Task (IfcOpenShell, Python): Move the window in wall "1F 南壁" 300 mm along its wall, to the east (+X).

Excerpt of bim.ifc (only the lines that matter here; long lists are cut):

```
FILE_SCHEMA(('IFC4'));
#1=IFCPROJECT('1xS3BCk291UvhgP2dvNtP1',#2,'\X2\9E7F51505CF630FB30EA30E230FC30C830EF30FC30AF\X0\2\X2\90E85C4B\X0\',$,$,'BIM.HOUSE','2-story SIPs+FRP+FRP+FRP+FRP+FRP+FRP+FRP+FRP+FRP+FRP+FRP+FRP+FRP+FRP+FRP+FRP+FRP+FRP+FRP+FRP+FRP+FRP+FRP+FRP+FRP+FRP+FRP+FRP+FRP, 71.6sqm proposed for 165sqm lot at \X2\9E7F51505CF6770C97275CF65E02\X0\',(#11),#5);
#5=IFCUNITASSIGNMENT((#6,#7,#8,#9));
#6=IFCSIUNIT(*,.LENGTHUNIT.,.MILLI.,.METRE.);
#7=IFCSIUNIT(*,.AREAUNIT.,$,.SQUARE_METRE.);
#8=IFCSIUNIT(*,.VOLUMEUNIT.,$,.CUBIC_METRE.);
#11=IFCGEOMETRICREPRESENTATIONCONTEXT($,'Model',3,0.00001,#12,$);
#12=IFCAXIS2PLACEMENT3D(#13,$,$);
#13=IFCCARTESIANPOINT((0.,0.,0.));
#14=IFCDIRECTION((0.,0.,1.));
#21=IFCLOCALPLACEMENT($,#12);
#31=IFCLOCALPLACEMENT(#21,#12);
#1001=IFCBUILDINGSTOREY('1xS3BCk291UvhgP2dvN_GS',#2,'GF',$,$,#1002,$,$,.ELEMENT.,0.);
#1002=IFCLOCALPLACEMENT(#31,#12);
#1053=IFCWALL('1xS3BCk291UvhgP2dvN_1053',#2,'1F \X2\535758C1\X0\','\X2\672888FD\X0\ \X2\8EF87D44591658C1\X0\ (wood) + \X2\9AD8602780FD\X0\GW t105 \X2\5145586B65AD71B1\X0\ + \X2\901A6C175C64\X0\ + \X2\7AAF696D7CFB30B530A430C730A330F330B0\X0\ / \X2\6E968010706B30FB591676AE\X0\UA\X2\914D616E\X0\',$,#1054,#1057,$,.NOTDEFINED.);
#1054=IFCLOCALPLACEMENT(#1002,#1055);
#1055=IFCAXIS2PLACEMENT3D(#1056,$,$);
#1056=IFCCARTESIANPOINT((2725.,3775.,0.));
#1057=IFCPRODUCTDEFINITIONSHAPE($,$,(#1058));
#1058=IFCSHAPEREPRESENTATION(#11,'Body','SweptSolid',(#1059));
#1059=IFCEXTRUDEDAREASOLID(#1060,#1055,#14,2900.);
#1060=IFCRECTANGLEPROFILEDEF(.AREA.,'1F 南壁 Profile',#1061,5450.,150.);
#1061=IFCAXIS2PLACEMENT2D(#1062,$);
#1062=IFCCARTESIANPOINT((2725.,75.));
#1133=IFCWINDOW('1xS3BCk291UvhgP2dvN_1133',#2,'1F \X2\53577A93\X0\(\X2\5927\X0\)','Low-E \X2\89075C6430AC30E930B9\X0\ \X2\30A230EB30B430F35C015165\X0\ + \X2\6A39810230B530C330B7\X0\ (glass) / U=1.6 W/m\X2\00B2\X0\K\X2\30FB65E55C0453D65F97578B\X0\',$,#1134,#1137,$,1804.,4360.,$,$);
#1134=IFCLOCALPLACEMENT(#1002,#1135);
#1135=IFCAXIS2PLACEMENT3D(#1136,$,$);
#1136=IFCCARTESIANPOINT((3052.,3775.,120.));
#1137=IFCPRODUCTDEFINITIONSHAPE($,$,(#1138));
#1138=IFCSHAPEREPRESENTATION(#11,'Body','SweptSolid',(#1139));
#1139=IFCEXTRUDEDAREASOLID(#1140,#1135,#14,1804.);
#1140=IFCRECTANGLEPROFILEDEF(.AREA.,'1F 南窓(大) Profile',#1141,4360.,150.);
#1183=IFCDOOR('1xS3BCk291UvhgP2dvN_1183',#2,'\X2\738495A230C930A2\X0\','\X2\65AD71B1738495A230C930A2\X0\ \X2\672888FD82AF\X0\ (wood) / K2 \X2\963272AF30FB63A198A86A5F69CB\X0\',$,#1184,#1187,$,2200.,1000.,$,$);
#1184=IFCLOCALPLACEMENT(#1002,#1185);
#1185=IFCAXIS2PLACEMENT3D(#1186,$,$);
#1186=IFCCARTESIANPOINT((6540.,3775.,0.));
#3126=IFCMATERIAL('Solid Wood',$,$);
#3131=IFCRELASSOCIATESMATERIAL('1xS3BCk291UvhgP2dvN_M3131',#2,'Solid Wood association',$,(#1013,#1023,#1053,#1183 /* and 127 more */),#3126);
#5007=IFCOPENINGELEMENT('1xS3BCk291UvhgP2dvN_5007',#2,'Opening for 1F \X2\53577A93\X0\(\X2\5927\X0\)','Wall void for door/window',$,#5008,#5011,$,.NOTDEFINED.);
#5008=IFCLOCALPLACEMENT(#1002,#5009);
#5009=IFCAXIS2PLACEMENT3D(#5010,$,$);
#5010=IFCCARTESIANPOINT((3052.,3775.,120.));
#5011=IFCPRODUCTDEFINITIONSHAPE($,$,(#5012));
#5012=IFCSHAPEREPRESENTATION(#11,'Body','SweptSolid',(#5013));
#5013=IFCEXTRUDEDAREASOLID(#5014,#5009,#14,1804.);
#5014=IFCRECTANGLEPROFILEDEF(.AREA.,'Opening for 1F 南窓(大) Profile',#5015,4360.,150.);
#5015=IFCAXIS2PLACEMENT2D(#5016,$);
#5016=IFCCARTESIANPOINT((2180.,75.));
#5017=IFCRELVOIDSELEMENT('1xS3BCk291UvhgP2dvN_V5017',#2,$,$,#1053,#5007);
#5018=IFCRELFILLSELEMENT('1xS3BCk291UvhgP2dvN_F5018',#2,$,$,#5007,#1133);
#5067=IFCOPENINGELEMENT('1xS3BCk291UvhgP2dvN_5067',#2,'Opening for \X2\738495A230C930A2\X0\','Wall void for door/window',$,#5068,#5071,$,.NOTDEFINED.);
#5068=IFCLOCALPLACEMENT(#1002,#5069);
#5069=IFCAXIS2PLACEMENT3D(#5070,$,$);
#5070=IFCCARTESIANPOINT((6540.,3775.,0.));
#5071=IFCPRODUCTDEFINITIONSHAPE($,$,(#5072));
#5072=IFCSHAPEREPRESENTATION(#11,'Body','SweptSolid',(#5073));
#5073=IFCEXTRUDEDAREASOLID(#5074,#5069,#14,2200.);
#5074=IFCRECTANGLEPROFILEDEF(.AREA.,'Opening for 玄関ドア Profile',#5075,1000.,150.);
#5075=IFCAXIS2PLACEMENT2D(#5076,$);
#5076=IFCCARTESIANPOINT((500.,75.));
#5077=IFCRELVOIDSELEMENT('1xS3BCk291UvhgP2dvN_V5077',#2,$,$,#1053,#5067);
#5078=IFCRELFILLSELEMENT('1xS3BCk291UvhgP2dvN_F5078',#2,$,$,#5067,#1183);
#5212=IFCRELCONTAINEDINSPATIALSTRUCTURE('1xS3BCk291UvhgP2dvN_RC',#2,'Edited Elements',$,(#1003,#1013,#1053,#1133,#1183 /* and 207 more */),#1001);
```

```python
import ifcopenshell
import ifcopenshell.api.geometry
import ifcopenshell.util.placement

model = ifcopenshell.open("bim.ifc")

window = model.by_guid("1xS3BCk291UvhgP2dvN_1133")
opening = window.FillsVoids[0].RelatingOpeningElement
wall = opening.VoidsElements[0].RelatingBuildingElement

wall_matrix = ifcopenshell.util.placement.get_local_placement(wall.ObjectPlacement)
shift = wall_matrix[:3, 0] * 300.0
before = ifcopenshell.util.placement.get_local_placement(window.ObjectPlacement)[:3, 3].copy()

# The window is not placed relative to its opening, so move both.
for product in (opening, window):
    matrix = ifcopenshell.util.placement.get_local_placement(product.ObjectPlacement)
    matrix[:3, 3] += shift
    ifcopenshell.api.geometry.edit_object_placement(model, product=product, matrix=matrix, is_si=False)

after = ifcopenshell.util.placement.get_local_placement(window.ObjectPlacement)[:3, 3]
print("window moved by", (after - before).round(3) + 0.0)

model.write("bim_edited.ifc")
```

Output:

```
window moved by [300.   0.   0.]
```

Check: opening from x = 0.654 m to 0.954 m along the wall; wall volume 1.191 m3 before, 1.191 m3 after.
